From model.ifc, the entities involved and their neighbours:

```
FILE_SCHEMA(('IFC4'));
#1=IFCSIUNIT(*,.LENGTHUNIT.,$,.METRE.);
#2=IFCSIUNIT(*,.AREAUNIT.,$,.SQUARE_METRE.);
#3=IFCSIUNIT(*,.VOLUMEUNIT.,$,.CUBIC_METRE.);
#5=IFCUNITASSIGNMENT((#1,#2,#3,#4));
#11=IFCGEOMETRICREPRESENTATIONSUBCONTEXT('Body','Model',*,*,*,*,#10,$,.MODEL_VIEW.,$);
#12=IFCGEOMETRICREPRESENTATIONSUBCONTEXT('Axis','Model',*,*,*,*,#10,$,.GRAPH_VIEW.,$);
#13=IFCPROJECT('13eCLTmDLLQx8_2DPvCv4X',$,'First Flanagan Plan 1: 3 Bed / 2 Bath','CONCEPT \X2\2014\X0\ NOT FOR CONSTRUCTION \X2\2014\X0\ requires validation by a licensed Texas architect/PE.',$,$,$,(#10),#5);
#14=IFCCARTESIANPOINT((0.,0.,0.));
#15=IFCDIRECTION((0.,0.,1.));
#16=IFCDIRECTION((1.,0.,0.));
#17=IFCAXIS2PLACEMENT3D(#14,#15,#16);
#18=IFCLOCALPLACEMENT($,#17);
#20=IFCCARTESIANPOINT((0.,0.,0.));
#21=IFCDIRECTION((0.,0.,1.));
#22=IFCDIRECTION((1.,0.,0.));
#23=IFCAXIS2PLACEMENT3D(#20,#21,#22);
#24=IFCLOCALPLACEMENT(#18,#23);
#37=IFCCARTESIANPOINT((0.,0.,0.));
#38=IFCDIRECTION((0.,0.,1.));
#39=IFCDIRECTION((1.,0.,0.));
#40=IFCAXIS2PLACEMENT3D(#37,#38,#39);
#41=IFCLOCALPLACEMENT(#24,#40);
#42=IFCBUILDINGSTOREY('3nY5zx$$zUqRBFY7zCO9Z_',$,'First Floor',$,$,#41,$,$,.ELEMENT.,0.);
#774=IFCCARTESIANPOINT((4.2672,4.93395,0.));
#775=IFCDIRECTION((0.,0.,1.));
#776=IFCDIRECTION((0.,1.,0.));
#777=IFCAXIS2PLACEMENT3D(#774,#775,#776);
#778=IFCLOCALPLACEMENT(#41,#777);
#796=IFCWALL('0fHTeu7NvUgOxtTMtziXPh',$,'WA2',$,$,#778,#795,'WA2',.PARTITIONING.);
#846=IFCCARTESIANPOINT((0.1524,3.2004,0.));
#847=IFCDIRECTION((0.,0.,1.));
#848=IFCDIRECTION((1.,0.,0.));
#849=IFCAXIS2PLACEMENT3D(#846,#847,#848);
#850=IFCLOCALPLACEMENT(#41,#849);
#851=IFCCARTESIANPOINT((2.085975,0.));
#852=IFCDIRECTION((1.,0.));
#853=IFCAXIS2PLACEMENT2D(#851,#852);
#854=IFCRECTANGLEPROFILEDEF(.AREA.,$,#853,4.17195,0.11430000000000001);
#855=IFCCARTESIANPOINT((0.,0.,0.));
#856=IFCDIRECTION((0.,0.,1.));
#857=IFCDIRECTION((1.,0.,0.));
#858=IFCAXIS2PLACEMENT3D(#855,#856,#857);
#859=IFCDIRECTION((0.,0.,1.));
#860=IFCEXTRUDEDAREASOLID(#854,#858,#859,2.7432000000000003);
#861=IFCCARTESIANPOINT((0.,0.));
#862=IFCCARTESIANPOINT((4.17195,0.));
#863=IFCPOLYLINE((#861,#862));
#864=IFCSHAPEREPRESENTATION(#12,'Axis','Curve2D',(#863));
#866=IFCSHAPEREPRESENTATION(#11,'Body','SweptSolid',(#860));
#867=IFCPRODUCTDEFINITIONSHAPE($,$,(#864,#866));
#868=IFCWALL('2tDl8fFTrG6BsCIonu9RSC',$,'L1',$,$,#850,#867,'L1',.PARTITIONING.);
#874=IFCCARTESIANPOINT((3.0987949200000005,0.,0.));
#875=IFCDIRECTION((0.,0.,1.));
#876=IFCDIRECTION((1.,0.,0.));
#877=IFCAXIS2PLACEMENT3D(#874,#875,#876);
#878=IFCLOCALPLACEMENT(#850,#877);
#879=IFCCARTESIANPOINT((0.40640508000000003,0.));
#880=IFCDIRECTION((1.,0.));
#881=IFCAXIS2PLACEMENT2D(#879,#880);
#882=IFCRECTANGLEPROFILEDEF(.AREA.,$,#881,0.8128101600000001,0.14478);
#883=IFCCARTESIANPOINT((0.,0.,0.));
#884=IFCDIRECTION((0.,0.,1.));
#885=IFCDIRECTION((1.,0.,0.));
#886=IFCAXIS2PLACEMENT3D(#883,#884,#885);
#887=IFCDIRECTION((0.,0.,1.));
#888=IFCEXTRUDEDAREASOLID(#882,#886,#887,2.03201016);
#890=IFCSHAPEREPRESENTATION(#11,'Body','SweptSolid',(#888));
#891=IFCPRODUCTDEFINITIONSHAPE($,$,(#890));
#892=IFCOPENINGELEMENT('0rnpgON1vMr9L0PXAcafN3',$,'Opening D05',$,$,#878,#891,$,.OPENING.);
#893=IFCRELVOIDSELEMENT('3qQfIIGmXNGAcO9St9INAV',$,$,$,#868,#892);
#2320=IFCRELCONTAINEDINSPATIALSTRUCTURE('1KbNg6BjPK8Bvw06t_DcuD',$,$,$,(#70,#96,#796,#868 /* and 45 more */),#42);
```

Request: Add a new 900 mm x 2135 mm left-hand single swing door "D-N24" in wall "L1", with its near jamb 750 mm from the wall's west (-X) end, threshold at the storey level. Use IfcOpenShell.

```python
import numpy as np
import ifcopenshell
import ifcopenshell.api.feature
import ifcopenshell.api.geometry
import ifcopenshell.api.root
import ifcopenshell.api.spatial
import ifcopenshell.geom
import ifcopenshell.util.element
import ifcopenshell.util.placement
import ifcopenshell.util.representation
import ifcopenshell.util.shape
import ifcopenshell.util.unit

model = ifcopenshell.open("model.ifc")
unit_scale = ifcopenshell.util.unit.calculate_unit_scale(model)
settings = ifcopenshell.geom.settings()


def volume(element):
    """Net volume in cubic metres, openings subtracted."""
    shape = ifcopenshell.geom.create_shape(settings, element)
    return ifcopenshell.util.shape.get_volume(shape.geometry)


wall = model.by_guid("2tDl8fFTrG6BsCIonu9RSC")
storey = ifcopenshell.util.element.get_container(wall, ifc_class="IfcBuildingStorey")
context = ifcopenshell.util.representation.get_context(model, "Model", "Body", "MODEL_VIEW")
before = volume(wall)

width, height, from_end, sill = 0.9, 2.135, 0.75, 0.0  # metres

# The wall runs along its own X axis, and the end named is its -X end.
wall_shape = ifcopenshell.geom.create_shape(settings, wall)
x, y, z = ifcopenshell.util.shape.get_vertices(wall_shape.geometry).T
start = x.min() + from_end
face, thickness = float(y.min()), float(y.max() - y.min())
wall_matrix = ifcopenshell.util.placement.get_local_placement(wall.ObjectPlacement)
level = ifcopenshell.util.placement.get_local_placement(storey.ObjectPlacement)[2, 3]


def in_wall(x, y):
    """Placement at x, y metres in the wall's axes, at sill height."""
    matrix = wall_matrix.copy()
    matrix[:, 3] = wall_matrix @ np.array([x / unit_scale, y / unit_scale, 0.0, 1.0])
    matrix[2, 3] = level + sill / unit_scale
    return matrix


# Opening: a box that overshoots both wall faces by 50 mm.
opening = ifcopenshell.api.root.create_entity(model, ifc_class="IfcOpeningElement", predefined_type="OPENING")
box = ifcopenshell.api.geometry.add_wall_representation(
    model, context=context, length=width, height=height, thickness=thickness + 0.1
)
ifcopenshell.api.geometry.assign_representation(model, product=opening, representation=box)
ifcopenshell.api.geometry.edit_object_placement(model, product=opening, matrix=in_wall(start, face - 0.05), is_si=False)
ifcopenshell.api.feature.add_feature(model, feature=opening, element=wall)

door = ifcopenshell.api.root.create_entity(model, ifc_class="IfcDoor", name="D-N24", predefined_type="DOOR")
door.OverallWidth, door.OverallHeight = width / unit_scale, height / unit_scale
door.OperationType = "SINGLE_SWING_LEFT"
body = ifcopenshell.api.geometry.add_door_representation(
    model,
    context=context,
    overall_width=door.OverallWidth,
    overall_height=door.OverallHeight,
    operation_type="SINGLE_SWING_LEFT",
    lining_properties={"LiningDepth": thickness / unit_scale, "ThresholdDepth": thickness / unit_scale},
)
ifcopenshell.api.geometry.assign_representation(model, product=door, representation=body)
ifcopenshell.api.spatial.assign_container(model, products=[door], relating_structure=storey)
ifcopenshell.api.feature.add_filling(model, opening=opening, element=door)

# The lining spans the wall, so the door starts at the wall face.
ifcopenshell.api.geometry.edit_object_placement(model, product=door, matrix=in_wall(start, face), is_si=False)

after = volume(wall)

print(f"wall volume {before:.3f} -> {after:.3f} m3")

model.write("model_v2.ifc")
```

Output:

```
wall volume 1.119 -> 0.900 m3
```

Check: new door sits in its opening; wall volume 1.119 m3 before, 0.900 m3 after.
